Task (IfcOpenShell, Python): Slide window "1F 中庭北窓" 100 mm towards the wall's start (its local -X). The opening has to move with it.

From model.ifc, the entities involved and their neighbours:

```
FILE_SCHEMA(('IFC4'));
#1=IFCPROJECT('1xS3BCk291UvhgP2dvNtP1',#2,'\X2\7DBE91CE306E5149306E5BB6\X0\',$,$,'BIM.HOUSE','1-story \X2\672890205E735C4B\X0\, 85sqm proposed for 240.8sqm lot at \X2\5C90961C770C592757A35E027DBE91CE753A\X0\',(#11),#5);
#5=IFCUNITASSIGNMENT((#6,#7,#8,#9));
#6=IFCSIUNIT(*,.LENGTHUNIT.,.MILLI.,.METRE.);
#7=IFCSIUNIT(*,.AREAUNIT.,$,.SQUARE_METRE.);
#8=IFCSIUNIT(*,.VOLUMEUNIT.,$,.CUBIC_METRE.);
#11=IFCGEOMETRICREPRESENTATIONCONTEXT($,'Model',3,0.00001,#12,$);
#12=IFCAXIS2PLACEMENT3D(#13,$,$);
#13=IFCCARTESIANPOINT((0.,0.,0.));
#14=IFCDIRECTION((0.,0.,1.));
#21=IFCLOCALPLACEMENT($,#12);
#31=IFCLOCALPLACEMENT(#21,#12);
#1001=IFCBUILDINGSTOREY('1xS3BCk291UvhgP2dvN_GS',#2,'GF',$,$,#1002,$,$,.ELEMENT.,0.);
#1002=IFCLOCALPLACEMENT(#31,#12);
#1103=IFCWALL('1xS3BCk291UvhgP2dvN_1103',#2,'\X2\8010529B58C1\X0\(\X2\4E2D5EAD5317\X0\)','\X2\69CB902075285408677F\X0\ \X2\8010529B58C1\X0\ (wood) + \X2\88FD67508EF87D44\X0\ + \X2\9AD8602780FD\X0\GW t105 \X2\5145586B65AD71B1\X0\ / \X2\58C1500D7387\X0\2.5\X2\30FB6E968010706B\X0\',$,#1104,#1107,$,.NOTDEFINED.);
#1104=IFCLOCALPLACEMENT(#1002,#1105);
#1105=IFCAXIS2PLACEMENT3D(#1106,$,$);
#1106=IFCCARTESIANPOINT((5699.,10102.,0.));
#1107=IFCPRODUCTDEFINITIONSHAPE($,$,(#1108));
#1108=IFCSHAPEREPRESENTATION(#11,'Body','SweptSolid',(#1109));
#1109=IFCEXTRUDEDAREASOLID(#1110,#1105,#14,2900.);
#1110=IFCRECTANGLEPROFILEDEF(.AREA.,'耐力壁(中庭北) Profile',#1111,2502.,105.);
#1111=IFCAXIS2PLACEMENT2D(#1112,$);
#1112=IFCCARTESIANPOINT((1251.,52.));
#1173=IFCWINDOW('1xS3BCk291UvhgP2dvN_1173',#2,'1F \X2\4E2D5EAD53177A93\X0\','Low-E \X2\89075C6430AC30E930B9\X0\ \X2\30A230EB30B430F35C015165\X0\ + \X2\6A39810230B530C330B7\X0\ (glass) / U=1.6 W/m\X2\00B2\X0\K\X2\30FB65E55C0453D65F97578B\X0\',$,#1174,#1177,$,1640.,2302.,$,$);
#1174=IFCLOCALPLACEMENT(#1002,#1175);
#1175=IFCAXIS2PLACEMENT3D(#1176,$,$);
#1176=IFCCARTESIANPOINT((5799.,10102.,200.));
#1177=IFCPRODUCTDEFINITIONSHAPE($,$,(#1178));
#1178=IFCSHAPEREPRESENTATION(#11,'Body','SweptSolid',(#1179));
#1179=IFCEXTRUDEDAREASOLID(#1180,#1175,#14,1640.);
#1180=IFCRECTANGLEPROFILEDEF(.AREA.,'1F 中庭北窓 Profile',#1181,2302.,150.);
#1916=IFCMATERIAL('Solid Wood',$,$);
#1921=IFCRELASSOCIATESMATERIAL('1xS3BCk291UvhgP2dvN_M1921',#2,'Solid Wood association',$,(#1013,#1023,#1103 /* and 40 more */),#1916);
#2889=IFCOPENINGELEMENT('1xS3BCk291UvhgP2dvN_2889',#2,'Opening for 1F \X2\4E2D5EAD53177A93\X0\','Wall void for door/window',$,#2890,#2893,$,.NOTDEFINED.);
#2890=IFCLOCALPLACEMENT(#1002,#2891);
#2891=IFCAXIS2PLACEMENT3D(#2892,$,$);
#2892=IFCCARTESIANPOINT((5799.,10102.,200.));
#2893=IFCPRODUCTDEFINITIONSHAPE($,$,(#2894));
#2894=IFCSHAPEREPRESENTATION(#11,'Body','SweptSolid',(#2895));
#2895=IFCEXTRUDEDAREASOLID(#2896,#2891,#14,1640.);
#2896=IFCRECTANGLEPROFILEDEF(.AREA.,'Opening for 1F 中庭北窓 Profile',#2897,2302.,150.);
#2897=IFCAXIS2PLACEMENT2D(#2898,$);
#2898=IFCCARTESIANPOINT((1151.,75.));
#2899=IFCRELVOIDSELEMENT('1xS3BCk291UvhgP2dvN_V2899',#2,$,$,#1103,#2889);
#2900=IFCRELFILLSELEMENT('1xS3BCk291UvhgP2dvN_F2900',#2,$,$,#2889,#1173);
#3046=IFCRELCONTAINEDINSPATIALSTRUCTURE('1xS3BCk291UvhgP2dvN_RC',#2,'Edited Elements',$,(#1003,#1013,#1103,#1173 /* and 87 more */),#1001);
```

```python
import ifcopenshell
import ifcopenshell.api.geometry
import ifcopenshell.util.placement

model = ifcopenshell.open("model.ifc")

window = model.by_guid("1xS3BCk291UvhgP2dvN_1173")
opening = window.FillsVoids[0].RelatingOpeningElement
wall = opening.VoidsElements[0].RelatingBuildingElement

wall_matrix = ifcopenshell.util.placement.get_local_placement(wall.ObjectPlacement)
shift = wall_matrix[:3, 0] * -100.0
before = ifcopenshell.util.placement.get_local_placement(window.ObjectPlacement)[:3, 3].copy()

# The window is not placed relative to its opening, so move both.
for product in (opening, window):
    matrix = ifcopenshell.util.placement.get_local_placement(product.ObjectPlacement)
    matrix[:3, 3] += shift
    ifcopenshell.api.geometry.edit_object_placement(model, product=product, matrix=matrix, is_si=False)

after = ifcopenshell.util.placement.get_local_placement(window.ObjectPlacement)[:3, 3]
print("window moved by", (after - before).round(3) + 0.0)

model.write("model_v2.ifc")
```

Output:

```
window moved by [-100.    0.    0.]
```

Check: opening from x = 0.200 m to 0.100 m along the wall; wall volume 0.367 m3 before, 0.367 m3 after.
